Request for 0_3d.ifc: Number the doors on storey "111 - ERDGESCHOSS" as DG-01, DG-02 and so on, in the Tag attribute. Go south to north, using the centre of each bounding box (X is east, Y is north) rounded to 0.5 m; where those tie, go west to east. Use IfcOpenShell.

First a look at what the model holds.

```python
import ifcopenshell
import ifcopenshell.util.element
import ifcopenshell.util.placement

model = ifcopenshell.open("0_3d.ifc")
print(model.schema)
storey = next(s for s in model.by_type("IfcBuildingStorey") if s.Name == "111 - ERDGESCHOSS")
doors = [e for e in ifcopenshell.util.element.get_decomposition(storey) if e.is_a("IfcDoor")]
for e in sorted(doors, key=lambda e: e.id()):
    origin = ifcopenshell.util.placement.get_local_placement(e.ObjectPlacement)[:3, 3]
    print(e.id(), e.Tag, e.Name, origin.round(2) + 0.0, sep=" | ")
```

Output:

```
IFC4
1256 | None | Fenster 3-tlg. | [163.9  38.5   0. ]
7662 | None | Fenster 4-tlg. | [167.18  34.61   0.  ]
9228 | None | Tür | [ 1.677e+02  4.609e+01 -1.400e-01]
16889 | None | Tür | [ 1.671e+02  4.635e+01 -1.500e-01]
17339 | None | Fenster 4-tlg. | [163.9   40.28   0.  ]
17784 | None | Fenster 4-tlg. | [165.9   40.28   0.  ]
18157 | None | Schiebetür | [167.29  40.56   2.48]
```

```python
import ifcopenshell
import ifcopenshell.geom
import ifcopenshell.util.element
import ifcopenshell.util.shape

model = ifcopenshell.open("0_3d.ifc")
settings = ifcopenshell.geom.settings()
settings.set("use-world-coords", True)


def centre(element):
    shape = ifcopenshell.geom.create_shape(settings, element)
    return ifcopenshell.util.shape.get_bbox_centroid(shape.geometry)


storey = next(s for s in model.by_type("IfcBuildingStorey") if s.Name == "111 - ERDGESCHOSS")
doors = [e for e in ifcopenshell.util.element.get_decomposition(storey) if e.is_a("IfcDoor")]

# Insertion points can sit at a corner or the storey origin, so sort by the geometry (in metres).
centres = {e: centre(e) for e in doors}
doors.sort(key=lambda e: (round(centres[e][1] / 0.5), centres[e][0]))

for i, e in enumerate(doors, start=1):
    number = f"DG-{i:02d}"
    e.Tag = number
    print(e.id(), number)

model.write("0_3d-out.ifc")
```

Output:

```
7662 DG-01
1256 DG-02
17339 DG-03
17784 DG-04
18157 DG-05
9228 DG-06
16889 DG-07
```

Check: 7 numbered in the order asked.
